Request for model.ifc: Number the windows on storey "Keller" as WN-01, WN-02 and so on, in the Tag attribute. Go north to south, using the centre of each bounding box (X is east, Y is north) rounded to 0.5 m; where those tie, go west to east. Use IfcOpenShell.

First a look at what the model holds.

```python
import ifcopenshell
import ifcopenshell.util.element
import ifcopenshell.util.placement

model = ifcopenshell.open("model.ifc")
print(model.schema)
storey = next(s for s in model.by_type("IfcBuildingStorey") if s.Name == "Keller")
windows = [e for e in ifcopenshell.util.element.get_decomposition(storey) if e.is_a("IfcWindow")]
for e in sorted(windows, key=lambda e: e.id()):
    origin = ifcopenshell.util.placement.get_local_placement(e.ObjectPlacement)[:3, 3]
    print(e.id(), e.Tag, e.Name, origin.round(2) + 0.0, sep=" | ")
```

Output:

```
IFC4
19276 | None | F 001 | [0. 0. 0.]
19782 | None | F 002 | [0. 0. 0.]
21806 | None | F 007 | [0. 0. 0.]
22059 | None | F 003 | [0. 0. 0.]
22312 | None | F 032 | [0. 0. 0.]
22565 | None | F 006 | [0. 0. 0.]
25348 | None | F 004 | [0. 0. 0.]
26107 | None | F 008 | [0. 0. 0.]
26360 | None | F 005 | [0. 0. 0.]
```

```python
import ifcopenshell
import ifcopenshell.geom
import ifcopenshell.util.element
import ifcopenshell.util.shape

model = ifcopenshell.open("model.ifc")
settings = ifcopenshell.geom.settings()
settings.set("use-world-coords", True)


def centre(element):
    shape = ifcopenshell.geom.create_shape(settings, element)
    return ifcopenshell.util.shape.get_bbox_centroid(shape.geometry)


storey = next(s for s in model.by_type("IfcBuildingStorey") if s.Name == "Keller")
windows = [e for e in ifcopenshell.util.element.get_decomposition(storey) if e.is_a("IfcWindow")]

# Insertion points can sit at a corner or the storey origin, so sort by the geometry (in metres).
centres = {e: centre(e) for e in windows}
windows.sort(key=lambda e: (-round(centres[e][1] / 0.5), centres[e][0]))

for i, e in enumerate(windows, start=1):
    number = f"WN-{i:02d}"
    e.Tag = number
    print(e.id(), number)

model.write("model-out.ifc")
```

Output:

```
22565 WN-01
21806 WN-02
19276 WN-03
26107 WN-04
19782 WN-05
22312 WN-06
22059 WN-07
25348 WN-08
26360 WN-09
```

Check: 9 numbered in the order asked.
